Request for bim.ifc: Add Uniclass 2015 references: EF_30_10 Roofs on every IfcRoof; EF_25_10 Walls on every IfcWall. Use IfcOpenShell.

First a look at what the model holds.

```python
import ifcopenshell

model = ifcopenshell.open("bim.ifc")
print(model.schema)
print("classifications:", [c.Name for c in model.by_type("IfcClassification")])
for ifc_class in ("IfcDoor", "IfcRoof", "IfcStair", "IfcWall", "IfcWindow"):
    print(ifc_class, len(model.by_type(ifc_class)))
```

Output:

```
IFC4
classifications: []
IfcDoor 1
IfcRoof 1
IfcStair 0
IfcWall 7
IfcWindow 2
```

```python
import ifcopenshell
import ifcopenshell.api.classification

model = ifcopenshell.open("bim.ifc")

system = ifcopenshell.api.classification.add_classification(model, classification="Uniclass 2015")

codes = {
    "IfcRoof": ("EF_30_10", "Roofs"),
    "IfcWall": ("EF_25_10", "Walls"),
}
for ifc_class, (code, name) in codes.items():
    products = model.by_type(ifc_class)
    ifcopenshell.api.classification.add_reference(
        model, products=products, classification=system, identification=code, name=name
    )
    print(code, len(products))

model.write("bim_updated.ifc")
```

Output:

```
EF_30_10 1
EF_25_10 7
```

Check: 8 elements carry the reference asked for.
